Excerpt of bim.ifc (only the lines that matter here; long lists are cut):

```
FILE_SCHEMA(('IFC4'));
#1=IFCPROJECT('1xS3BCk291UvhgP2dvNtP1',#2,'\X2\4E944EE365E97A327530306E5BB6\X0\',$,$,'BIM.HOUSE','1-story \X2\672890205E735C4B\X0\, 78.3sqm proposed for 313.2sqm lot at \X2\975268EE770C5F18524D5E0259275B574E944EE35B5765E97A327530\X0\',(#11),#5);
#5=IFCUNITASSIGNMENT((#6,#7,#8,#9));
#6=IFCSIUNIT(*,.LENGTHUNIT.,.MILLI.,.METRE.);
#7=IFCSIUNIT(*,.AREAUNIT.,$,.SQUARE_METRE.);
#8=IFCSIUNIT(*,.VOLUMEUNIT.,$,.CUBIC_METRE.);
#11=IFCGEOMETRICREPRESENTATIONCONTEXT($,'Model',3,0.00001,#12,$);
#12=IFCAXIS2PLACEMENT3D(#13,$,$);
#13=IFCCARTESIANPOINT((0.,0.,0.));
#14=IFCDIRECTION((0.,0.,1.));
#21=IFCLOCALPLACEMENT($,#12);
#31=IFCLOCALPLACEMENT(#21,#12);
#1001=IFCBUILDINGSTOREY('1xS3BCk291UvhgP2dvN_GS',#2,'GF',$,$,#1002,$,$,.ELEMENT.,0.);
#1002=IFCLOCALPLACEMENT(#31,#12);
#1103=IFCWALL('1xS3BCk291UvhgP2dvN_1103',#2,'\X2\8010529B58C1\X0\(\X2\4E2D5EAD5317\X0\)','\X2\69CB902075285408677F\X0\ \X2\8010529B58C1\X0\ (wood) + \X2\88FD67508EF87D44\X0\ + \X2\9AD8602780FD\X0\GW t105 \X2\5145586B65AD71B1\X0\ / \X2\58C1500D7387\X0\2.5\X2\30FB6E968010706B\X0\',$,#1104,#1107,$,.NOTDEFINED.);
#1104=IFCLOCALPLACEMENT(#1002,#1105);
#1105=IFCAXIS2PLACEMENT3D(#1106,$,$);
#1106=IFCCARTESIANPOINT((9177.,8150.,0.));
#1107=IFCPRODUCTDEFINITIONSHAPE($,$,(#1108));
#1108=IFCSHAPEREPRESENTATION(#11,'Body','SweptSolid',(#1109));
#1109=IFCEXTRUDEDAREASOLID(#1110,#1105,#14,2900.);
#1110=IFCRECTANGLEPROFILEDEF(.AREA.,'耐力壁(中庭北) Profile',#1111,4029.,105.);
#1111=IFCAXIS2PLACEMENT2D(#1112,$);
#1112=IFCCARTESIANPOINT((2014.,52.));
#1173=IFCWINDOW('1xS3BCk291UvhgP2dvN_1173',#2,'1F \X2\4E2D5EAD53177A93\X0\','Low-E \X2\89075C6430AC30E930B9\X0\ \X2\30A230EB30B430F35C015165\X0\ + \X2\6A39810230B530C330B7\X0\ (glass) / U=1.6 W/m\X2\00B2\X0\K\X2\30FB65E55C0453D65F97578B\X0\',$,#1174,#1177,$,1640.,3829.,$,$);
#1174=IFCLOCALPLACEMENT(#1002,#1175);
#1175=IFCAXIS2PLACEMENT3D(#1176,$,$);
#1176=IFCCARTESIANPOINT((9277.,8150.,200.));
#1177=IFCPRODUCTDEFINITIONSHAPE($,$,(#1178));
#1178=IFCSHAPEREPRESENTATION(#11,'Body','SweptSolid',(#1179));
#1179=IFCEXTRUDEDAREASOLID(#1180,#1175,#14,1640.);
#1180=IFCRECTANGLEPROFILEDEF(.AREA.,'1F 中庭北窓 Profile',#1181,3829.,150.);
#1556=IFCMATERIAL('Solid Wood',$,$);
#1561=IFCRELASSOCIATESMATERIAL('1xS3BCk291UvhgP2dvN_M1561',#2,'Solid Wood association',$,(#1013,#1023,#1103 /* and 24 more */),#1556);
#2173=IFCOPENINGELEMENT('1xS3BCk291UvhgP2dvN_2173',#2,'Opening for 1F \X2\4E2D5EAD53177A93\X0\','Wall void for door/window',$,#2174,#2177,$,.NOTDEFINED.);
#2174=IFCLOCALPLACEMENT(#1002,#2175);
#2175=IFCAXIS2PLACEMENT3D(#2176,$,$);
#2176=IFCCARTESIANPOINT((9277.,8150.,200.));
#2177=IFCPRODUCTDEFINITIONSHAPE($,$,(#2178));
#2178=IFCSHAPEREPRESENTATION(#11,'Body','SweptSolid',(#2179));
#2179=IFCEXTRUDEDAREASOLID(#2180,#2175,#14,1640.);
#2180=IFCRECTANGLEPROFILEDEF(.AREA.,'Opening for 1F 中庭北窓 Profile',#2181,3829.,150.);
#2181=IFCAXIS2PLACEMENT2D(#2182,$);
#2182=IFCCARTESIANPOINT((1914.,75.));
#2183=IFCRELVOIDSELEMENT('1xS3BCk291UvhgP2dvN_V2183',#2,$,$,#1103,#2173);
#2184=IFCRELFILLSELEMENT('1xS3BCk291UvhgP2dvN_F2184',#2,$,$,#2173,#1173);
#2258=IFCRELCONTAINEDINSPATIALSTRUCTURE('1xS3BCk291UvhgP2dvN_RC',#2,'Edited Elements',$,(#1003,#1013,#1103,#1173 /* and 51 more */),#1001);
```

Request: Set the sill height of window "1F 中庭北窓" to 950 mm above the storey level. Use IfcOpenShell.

```python
import numpy as np
import ifcopenshell
import ifcopenshell.api.geometry
import ifcopenshell.geom
import ifcopenshell.util.element
import ifcopenshell.util.placement
import ifcopenshell.util.shape
import ifcopenshell.util.unit

model = ifcopenshell.open("bim.ifc")
unit_scale = ifcopenshell.util.unit.calculate_unit_scale(model)

window = model.by_id(1173)
opening = window.FillsVoids[0].RelatingOpeningElement
storey = ifcopenshell.util.element.get_container(window, ifc_class="IfcBuildingStorey")
level = ifcopenshell.util.placement.get_local_placement(storey.ObjectPlacement)[2, 3]

# The opening's origin need not be at the sill, so measure its lowest point.
shape = ifcopenshell.geom.create_shape(ifcopenshell.geom.settings(), opening)
bottom = ifcopenshell.util.shape.get_shape_bottom_elevation(shape, shape.geometry) / unit_scale
dz = level + 0.95 / unit_scale - bottom

shift = np.array([0.0, 0.0, dz])
# The window is not placed relative to its opening, so move both.
for product in (opening, window):
    matrix = ifcopenshell.util.placement.get_local_placement(product.ObjectPlacement)
    matrix[:3, 3] += shift
    ifcopenshell.api.geometry.edit_object_placement(model, product=product, matrix=matrix, is_si=False)

print(f"moved by {dz * unit_scale:+.3f} m")

model.write("bim_v2.ifc")
```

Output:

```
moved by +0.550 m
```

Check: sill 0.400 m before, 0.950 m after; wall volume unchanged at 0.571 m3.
